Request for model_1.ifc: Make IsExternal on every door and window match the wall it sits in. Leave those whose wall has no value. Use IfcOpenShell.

First a look at what the model holds.

```python
import ifcopenshell
import ifcopenshell.util.element

model = ifcopenshell.open("model_1.ifc")
print(model.schema)
seen = {}
for e in model.by_type("IfcDoor") + model.by_type("IfcWindow"):
    if not e.FillsVoids:
        continue
    host = e.FillsVoids[0].RelatingOpeningElement.VoidsElements[0].RelatingBuildingElement
    own = ifcopenshell.util.element.get_pset(e, f"Pset_{e.is_a()[3:].removesuffix('StandardCase')}Common", "IsExternal")
    wall = ifcopenshell.util.element.get_pset(host, "Pset_WallCommon", "IsExternal")
    seen[e.is_a(), own, wall] = seen.get((e.is_a(), own, wall), 0) + 1
for (cls, own, wall), count in sorted(seen.items(), key=str):
    print(count, cls, "IsExternal:", own, "| host wall:", wall)
```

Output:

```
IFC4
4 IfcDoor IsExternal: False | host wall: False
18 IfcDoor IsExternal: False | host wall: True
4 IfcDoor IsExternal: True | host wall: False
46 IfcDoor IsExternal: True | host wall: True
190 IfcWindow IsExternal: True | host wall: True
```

```python
import ifcopenshell
import ifcopenshell.api.pset
import ifcopenshell.util.element

model = ifcopenshell.open("model_1.ifc")

count = 0
for ifc_class, pset_name in (("IfcDoor", "Pset_DoorCommon"), ("IfcWindow", "Pset_WindowCommon")):
    for e in model.by_type(ifc_class):
        if not e.FillsVoids:
            continue
        host = e.FillsVoids[0].RelatingOpeningElement.VoidsElements[0].RelatingBuildingElement
        external = ifcopenshell.util.element.get_pset(host, "Pset_WallCommon", "IsExternal")
        if external is None or ifcopenshell.util.element.get_pset(e, pset_name, "IsExternal") == external:
            continue
        pset = ifcopenshell.api.pset.add_pset(model, product=e, name=pset_name)
        ifcopenshell.api.pset.edit_pset(model, pset=pset, properties={"IsExternal": external})
        count += 1

print(count, "updated")

model.write("model_1_v2.ifc")
```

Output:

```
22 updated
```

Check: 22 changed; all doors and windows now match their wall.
